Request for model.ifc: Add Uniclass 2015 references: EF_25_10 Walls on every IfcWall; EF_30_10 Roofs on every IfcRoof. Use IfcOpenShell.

First a look at what the model holds.

```python
import ifcopenshell

model = ifcopenshell.open("model.ifc")
print(model.schema)
print("classifications:", [c.Name for c in model.by_type("IfcClassification")])
for ifc_class in ("IfcDoor", "IfcRoof", "IfcStair", "IfcWall", "IfcWindow"):
    print(ifc_class, len(model.by_type(ifc_class)))
```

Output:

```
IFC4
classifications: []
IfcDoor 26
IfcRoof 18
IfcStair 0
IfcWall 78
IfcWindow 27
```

```python
import ifcopenshell
import ifcopenshell.api.classification

model = ifcopenshell.open("model.ifc")

system = ifcopenshell.api.classification.add_classification(model, classification="Uniclass 2015")

codes = {
    "IfcWall": ("EF_25_10", "Walls"),
    "IfcRoof": ("EF_30_10", "Roofs"),
}
for ifc_class, (code, name) in codes.items():
    products = model.by_type(ifc_class)
    ifcopenshell.api.classification.add_reference(
        model, products=products, classification=system, identification=code, name=name
    )
    print(code, len(products))

model.write("model_edited.ifc")
```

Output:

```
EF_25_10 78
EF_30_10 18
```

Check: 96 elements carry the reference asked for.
